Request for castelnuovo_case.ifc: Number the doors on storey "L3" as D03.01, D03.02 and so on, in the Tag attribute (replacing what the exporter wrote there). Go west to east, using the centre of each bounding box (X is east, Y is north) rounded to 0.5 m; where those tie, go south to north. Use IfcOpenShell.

First a look at what the model holds.

```python
import ifcopenshell
import ifcopenshell.util.element
import ifcopenshell.util.placement

model = ifcopenshell.open("castelnuovo_case.ifc")
print(model.schema)
storey = next(s for s in model.by_type("IfcBuildingStorey") if s.Name == "L3")
doors = [e for e in ifcopenshell.util.element.get_decomposition(storey) if e.is_a("IfcDoor")]
for e in sorted(doors, key=lambda e: e.id()):
    origin = ifcopenshell.util.placement.get_local_placement(e.ObjectPlacement)[:3, 3]
    print(e.id(), e.Tag, e.Name, origin.round(2) + 0.0, sep=" | ")
```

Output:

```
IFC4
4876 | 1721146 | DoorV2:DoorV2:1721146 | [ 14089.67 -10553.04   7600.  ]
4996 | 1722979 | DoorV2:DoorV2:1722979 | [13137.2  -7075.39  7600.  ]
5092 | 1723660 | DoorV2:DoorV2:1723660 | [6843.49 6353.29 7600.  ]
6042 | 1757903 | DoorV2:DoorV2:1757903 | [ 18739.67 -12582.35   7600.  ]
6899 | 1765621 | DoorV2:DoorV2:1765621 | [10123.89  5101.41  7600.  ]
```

```python
import ifcopenshell
import ifcopenshell.geom
import ifcopenshell.util.element
import ifcopenshell.util.shape

model = ifcopenshell.open("castelnuovo_case.ifc")
settings = ifcopenshell.geom.settings()
settings.set("use-world-coords", True)


def centre(element):
    shape = ifcopenshell.geom.create_shape(settings, element)
    return ifcopenshell.util.shape.get_bbox_centroid(shape.geometry)


storey = next(s for s in model.by_type("IfcBuildingStorey") if s.Name == "L3")
doors = [e for e in ifcopenshell.util.element.get_decomposition(storey) if e.is_a("IfcDoor")]

# Insertion points can sit at a corner or the storey origin, so sort by the geometry (in metres).
centres = {e: centre(e) for e in doors}
doors.sort(key=lambda e: (round(centres[e][0] / 0.5), centres[e][1]))

for i, e in enumerate(doors, start=1):
    number = f"D03.{i:02d}"
    e.Tag = number
    print(e.id(), number)

model.write("castelnuovo_case-out.ifc")
```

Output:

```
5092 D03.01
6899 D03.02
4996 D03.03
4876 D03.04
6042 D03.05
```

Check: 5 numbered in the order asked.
